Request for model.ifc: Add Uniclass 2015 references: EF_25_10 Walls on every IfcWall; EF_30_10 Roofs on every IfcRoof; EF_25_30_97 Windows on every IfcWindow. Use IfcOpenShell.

First a look at what the model holds.

```python
import ifcopenshell

model = ifcopenshell.open("model.ifc")
print(model.schema)
print("classifications:", [c.Name for c in model.by_type("IfcClassification")])
for ifc_class in ("IfcDoor", "IfcRoof", "IfcStair", "IfcWall", "IfcWindow"):
    print(ifc_class, len(model.by_type(ifc_class)))
```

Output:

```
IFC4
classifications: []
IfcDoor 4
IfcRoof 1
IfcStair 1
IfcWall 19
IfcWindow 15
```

```python
import ifcopenshell
import ifcopenshell.api.classification

model = ifcopenshell.open("model.ifc")

system = ifcopenshell.api.classification.add_classification(model, classification="Uniclass 2015")

codes = {
    "IfcWall": ("EF_25_10", "Walls"),
    "IfcRoof": ("EF_30_10", "Roofs"),
    "IfcWindow": ("EF_25_30_97", "Windows"),
}
for ifc_class, (code, name) in codes.items():
    products = model.by_type(ifc_class)
    ifcopenshell.api.classification.add_reference(
        model, products=products, classification=system, identification=code, name=name
    )
    print(code, len(products))

model.write("model_rev.ifc")
```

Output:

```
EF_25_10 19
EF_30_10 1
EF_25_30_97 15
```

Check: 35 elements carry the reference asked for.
